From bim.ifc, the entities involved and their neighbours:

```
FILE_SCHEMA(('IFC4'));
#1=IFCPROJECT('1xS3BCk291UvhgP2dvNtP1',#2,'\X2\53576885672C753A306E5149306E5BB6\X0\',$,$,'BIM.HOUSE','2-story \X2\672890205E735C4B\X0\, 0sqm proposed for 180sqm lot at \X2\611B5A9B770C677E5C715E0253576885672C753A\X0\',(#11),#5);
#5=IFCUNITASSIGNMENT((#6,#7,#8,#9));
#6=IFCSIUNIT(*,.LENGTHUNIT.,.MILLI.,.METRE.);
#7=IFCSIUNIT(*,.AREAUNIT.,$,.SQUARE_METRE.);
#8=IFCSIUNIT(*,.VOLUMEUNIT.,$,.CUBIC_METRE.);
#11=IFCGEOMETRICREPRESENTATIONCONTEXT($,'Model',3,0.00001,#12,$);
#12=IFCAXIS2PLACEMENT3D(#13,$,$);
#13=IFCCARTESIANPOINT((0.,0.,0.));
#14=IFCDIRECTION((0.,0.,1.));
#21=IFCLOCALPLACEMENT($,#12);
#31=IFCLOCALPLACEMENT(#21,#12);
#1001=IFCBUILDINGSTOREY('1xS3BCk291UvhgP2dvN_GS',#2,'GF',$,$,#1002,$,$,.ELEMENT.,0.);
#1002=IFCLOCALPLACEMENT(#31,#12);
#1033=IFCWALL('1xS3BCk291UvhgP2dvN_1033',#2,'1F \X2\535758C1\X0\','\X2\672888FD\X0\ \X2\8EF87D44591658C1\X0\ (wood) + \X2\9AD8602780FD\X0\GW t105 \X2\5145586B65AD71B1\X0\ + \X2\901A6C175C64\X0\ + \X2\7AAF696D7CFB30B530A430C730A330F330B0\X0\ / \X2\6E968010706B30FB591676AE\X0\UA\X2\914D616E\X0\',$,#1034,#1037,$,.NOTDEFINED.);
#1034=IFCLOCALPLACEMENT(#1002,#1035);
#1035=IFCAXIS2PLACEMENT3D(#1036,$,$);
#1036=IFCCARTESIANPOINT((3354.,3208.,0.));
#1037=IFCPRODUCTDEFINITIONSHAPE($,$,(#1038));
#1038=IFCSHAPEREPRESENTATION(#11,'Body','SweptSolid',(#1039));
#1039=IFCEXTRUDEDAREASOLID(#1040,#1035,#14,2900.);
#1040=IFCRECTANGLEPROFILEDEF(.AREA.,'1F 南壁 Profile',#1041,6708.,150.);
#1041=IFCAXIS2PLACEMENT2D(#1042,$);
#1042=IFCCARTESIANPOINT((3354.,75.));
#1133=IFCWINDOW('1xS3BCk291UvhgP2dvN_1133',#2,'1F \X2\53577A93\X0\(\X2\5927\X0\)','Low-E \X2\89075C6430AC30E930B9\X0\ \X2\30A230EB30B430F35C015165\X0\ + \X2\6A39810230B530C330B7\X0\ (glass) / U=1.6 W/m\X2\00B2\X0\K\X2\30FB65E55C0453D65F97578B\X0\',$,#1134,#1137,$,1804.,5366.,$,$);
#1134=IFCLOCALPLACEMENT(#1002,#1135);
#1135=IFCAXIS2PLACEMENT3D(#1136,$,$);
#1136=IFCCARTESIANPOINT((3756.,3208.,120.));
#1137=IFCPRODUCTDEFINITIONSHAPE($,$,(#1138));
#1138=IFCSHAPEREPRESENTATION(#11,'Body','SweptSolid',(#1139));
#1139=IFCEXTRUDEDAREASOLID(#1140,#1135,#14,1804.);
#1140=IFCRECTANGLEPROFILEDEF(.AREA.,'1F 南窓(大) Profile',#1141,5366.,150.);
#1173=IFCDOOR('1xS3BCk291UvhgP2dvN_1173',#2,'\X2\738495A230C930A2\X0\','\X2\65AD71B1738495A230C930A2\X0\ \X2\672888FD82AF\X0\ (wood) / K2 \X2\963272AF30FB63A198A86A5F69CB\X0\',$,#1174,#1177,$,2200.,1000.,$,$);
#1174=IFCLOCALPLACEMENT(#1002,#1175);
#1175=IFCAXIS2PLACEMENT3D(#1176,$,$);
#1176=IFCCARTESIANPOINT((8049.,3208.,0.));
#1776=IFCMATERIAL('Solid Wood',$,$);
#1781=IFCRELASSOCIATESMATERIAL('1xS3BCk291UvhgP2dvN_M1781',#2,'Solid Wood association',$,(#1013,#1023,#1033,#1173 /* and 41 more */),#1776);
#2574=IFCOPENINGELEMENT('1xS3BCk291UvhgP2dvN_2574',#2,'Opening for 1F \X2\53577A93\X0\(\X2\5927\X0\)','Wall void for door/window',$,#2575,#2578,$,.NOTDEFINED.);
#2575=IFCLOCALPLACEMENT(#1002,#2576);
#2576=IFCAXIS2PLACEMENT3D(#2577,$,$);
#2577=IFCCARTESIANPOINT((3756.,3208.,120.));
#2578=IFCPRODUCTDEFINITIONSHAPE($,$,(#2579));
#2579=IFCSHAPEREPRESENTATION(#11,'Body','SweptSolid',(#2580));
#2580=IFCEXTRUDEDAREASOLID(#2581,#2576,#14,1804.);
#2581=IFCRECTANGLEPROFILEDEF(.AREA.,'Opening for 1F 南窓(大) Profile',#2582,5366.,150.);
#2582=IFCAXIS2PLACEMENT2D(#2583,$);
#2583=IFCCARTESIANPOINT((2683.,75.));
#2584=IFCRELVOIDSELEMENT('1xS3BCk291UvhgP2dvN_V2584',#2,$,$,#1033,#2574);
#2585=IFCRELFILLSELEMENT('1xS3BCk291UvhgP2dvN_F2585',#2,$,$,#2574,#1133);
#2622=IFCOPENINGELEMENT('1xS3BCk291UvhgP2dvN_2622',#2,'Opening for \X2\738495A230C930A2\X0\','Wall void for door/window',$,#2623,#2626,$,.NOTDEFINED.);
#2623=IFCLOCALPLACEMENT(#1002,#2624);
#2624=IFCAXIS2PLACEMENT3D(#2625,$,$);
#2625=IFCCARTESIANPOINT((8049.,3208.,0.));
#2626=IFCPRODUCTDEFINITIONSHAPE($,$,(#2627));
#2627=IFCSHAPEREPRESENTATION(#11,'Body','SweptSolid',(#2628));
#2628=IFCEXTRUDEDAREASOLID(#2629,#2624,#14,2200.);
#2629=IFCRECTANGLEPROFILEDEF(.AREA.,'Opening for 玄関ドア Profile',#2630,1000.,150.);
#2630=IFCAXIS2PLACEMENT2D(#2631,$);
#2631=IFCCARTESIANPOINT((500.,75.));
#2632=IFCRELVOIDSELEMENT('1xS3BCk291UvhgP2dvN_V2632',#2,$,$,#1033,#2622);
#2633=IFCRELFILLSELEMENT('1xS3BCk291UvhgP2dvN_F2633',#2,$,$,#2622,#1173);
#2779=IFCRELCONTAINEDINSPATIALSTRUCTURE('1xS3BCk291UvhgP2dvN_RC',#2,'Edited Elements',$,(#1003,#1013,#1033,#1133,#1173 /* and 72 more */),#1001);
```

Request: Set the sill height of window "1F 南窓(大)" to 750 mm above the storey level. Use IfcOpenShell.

```python
import numpy as np
import ifcopenshell
import ifcopenshell.api.geometry
import ifcopenshell.geom
import ifcopenshell.util.element
import ifcopenshell.util.placement
import ifcopenshell.util.shape
import ifcopenshell.util.unit

model = ifcopenshell.open("bim.ifc")
unit_scale = ifcopenshell.util.unit.calculate_unit_scale(model)

window = model.by_id(1133)
opening = window.FillsVoids[0].RelatingOpeningElement
storey = ifcopenshell.util.element.get_container(window, ifc_class="IfcBuildingStorey")
level = ifcopenshell.util.placement.get_local_placement(storey.ObjectPlacement)[2, 3]

# The opening's origin need not be at the sill, so measure its lowest point.
shape = ifcopenshell.geom.create_shape(ifcopenshell.geom.settings(), opening)
bottom = ifcopenshell.util.shape.get_shape_bottom_elevation(shape, shape.geometry) / unit_scale
dz = level + 750.0 - bottom

shift = np.array([0.0, 0.0, dz])
# The window is not placed relative to its opening, so move both.
for product in (opening, window):
    matrix = ifcopenshell.util.placement.get_local_placement(product.ObjectPlacement)
    matrix[:3, 3] += shift
    ifcopenshell.api.geometry.edit_object_placement(model, product=product, matrix=matrix, is_si=False)

print(f"moved by {dz * unit_scale:+.3f} m")

model.write("bim_v2.ifc")
```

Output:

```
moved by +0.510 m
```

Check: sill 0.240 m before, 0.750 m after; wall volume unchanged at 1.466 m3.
